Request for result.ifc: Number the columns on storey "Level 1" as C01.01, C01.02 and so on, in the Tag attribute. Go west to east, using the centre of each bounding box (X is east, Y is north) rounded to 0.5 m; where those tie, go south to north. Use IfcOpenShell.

First a look at what the model holds.

```python
import ifcopenshell
import ifcopenshell.util.element
import ifcopenshell.util.placement

model = ifcopenshell.open("result.ifc")
print(model.schema)
storey = next(s for s in model.by_type("IfcBuildingStorey") if s.Name == "Level 1")
columns = [e for e in ifcopenshell.util.element.get_decomposition(storey) if e.is_a("IfcColumn")]
for e in sorted(columns, key=lambda e: e.id()):
    origin = ifcopenshell.util.placement.get_local_placement(e.ObjectPlacement)[:3, 3]
    print(e.id(), e.Tag, e.Name, origin.round(2) + 0.0, sep=" | ")
```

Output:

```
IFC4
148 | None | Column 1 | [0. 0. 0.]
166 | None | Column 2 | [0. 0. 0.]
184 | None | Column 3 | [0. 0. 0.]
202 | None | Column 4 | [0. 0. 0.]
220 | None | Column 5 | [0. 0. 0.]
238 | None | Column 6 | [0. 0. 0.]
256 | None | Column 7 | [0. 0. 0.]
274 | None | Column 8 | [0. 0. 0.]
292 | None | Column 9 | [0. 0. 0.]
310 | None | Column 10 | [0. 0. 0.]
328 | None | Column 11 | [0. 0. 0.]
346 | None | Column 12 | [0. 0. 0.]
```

```python
import ifcopenshell
import ifcopenshell.geom
import ifcopenshell.util.element
import ifcopenshell.util.shape

model = ifcopenshell.open("result.ifc")
settings = ifcopenshell.geom.settings()
settings.set("use-world-coords", True)


def centre(element):
    shape = ifcopenshell.geom.create_shape(settings, element)
    return ifcopenshell.util.shape.get_bbox_centroid(shape.geometry)


storey = next(s for s in model.by_type("IfcBuildingStorey") if s.Name == "Level 1")
columns = [e for e in ifcopenshell.util.element.get_decomposition(storey) if e.is_a("IfcColumn")]

# Insertion points can sit at a corner or the storey origin, so sort by the geometry (in metres).
centres = {e: centre(e) for e in columns}
columns.sort(key=lambda e: (round(centres[e][0] / 0.5), centres[e][1]))

for i, e in enumerate(columns, start=1):
    number = f"C01.{i:02d}"
    e.Tag = number
    print(e.id(), number)

model.write("result-out.ifc")
```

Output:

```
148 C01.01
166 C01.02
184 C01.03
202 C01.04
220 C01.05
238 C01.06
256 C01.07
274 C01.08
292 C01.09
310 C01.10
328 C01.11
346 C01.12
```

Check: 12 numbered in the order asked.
